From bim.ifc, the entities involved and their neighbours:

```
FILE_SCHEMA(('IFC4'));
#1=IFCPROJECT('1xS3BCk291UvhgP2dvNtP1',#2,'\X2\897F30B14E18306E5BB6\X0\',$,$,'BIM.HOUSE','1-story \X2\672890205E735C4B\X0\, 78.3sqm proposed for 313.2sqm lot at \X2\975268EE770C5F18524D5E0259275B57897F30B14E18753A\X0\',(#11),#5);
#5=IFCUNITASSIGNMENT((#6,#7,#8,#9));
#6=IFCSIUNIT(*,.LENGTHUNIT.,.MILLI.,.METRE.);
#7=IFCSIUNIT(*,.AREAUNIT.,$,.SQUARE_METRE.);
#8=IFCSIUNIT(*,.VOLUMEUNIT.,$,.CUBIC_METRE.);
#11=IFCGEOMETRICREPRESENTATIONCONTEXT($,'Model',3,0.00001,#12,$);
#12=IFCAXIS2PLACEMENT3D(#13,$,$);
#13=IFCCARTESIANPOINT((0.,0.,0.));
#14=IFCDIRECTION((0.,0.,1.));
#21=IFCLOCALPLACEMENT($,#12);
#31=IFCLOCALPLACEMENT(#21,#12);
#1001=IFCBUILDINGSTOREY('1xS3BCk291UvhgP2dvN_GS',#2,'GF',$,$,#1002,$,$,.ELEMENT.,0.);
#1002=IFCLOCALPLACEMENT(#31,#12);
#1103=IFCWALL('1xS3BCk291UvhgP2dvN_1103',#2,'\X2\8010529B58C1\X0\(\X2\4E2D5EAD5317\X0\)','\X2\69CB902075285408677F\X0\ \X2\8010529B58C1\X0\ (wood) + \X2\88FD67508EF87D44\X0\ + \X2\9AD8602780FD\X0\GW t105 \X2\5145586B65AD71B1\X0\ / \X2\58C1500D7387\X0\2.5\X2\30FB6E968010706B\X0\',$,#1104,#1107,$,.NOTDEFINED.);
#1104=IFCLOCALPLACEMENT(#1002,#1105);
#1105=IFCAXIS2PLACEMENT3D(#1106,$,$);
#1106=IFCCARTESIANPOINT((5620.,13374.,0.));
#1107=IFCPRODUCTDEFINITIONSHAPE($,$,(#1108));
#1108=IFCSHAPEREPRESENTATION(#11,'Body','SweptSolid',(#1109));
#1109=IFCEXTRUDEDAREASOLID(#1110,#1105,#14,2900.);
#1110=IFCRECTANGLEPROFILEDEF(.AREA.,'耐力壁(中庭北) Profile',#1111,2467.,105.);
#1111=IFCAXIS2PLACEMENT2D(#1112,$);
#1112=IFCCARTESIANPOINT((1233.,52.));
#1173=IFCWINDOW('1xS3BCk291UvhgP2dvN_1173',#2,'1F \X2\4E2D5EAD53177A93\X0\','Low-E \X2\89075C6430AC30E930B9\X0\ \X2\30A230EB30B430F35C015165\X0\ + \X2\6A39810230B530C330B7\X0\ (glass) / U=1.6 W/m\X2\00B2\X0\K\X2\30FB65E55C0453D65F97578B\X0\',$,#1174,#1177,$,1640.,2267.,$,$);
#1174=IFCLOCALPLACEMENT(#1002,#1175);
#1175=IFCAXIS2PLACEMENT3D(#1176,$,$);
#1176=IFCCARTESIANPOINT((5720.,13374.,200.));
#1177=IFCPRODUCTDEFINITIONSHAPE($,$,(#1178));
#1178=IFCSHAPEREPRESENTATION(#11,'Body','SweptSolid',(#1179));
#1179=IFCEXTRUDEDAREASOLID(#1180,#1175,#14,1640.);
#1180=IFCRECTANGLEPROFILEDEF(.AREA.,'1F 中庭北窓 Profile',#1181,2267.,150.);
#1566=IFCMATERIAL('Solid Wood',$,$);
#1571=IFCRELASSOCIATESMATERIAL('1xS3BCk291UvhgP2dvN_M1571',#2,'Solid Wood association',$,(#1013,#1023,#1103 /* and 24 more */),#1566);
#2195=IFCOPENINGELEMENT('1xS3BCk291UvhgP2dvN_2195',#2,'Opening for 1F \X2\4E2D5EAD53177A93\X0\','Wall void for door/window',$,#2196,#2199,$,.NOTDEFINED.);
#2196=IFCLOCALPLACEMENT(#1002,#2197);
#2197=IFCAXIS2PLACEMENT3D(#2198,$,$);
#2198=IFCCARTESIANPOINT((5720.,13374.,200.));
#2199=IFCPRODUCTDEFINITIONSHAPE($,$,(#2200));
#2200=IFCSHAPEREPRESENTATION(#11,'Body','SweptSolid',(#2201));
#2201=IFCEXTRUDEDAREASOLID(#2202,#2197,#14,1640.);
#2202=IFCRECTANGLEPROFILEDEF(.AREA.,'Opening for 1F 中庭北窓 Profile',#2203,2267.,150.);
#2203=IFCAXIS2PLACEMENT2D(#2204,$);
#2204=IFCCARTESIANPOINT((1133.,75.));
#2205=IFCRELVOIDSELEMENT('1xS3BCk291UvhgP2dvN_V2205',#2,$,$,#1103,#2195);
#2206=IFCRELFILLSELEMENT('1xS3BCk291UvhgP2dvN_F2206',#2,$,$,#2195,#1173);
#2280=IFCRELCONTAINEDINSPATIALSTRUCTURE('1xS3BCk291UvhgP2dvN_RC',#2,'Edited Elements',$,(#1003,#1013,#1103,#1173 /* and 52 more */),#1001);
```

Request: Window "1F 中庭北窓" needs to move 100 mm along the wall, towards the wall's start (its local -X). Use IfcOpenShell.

```python
import ifcopenshell
import ifcopenshell.api.geometry
import ifcopenshell.util.placement

model = ifcopenshell.open("bim.ifc")

window = model.by_guid("1xS3BCk291UvhgP2dvN_1173")
opening = window.FillsVoids[0].RelatingOpeningElement
wall = opening.VoidsElements[0].RelatingBuildingElement

wall_matrix = ifcopenshell.util.placement.get_local_placement(wall.ObjectPlacement)
shift = wall_matrix[:3, 0] * -100.0
before = ifcopenshell.util.placement.get_local_placement(window.ObjectPlacement)[:3, 3].copy()

# The window is not placed relative to its opening, so move both.
for product in (opening, window):
    matrix = ifcopenshell.util.placement.get_local_placement(product.ObjectPlacement)
    matrix[:3, 3] += shift
    ifcopenshell.api.geometry.edit_object_placement(model, product=product, matrix=matrix, is_si=False)

after = ifcopenshell.util.placement.get_local_placement(window.ObjectPlacement)[:3, 3]
print("window moved by", (after - before).round(3) + 0.0)

model.write("bim_updated.ifc")
```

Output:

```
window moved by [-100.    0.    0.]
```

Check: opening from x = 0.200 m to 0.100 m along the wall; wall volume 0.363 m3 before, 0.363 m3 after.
